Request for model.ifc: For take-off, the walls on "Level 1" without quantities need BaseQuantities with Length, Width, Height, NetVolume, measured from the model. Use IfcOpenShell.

First a look at what the model holds.

```python
import ifcopenshell
import ifcopenshell.util.element
import ifcopenshell.util.unit

model = ifcopenshell.open("model.ifc")
print(model.schema)
for unit_type in ("LENGTHUNIT", "AREAUNIT", "VOLUMEUNIT"):
    print(unit_type, ifcopenshell.util.unit.calculate_unit_scale(model, unit_type))
storey = next(s for s in model.by_type("IfcBuildingStorey") if s.Name == "Level 1")
walls = [e for e in ifcopenshell.util.element.get_decomposition(storey) if e.is_a("IfcWall")]
for e in sorted(walls, key=lambda e: e.id()):
    print(e.id(), e.is_a(), e.Name, list(ifcopenshell.util.element.get_psets(e, qtos_only=True)), sep=" | ")
```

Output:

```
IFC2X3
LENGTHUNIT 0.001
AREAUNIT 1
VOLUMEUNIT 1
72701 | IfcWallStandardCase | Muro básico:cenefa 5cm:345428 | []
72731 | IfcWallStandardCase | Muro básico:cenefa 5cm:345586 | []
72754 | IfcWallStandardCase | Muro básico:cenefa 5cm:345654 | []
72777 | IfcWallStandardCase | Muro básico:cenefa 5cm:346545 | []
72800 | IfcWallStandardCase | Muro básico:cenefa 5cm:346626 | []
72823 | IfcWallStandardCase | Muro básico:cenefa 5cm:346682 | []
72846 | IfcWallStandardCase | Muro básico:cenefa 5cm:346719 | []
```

```python
import ifcopenshell
import ifcopenshell.api.pset
import ifcopenshell.geom
import ifcopenshell.util.element
import ifcopenshell.util.shape
import ifcopenshell.util.unit

model = ifcopenshell.open("model.ifc")
unit_scale = ifcopenshell.util.unit.calculate_unit_scale(model)
volume_scale = ifcopenshell.util.unit.calculate_unit_scale(model, "VOLUMEUNIT")
settings = ifcopenshell.geom.settings()

storey = next(s for s in model.by_type("IfcBuildingStorey") if s.Name == "Level 1")
walls = [e for e in ifcopenshell.util.element.get_decomposition(storey) if e.is_a("IfcWall")]

for e in sorted(walls, key=lambda e: e.id()):
    if ifcopenshell.util.element.get_psets(e, qtos_only=True, should_inherit=False):
        continue
    # Geometry comes back in metres, in the element's own axes.
    shape = ifcopenshell.geom.create_shape(settings, e)
    values = {
        "Length": ifcopenshell.util.shape.get_x(shape.geometry) / unit_scale,
        "Width": ifcopenshell.util.shape.get_y(shape.geometry) / unit_scale,
        "Height": ifcopenshell.util.shape.get_z(shape.geometry) / unit_scale,
        "NetVolume": ifcopenshell.util.shape.get_volume(shape.geometry) / volume_scale,
    }
    qto = ifcopenshell.api.pset.add_qto(model, product=e, name="BaseQuantities")
    ifcopenshell.api.pset.edit_qto(model, qto=qto, properties=values)
    print(e.id(), {k: round(v, 3) for k, v in values.items()})

model.write("model_v2.ifc")
```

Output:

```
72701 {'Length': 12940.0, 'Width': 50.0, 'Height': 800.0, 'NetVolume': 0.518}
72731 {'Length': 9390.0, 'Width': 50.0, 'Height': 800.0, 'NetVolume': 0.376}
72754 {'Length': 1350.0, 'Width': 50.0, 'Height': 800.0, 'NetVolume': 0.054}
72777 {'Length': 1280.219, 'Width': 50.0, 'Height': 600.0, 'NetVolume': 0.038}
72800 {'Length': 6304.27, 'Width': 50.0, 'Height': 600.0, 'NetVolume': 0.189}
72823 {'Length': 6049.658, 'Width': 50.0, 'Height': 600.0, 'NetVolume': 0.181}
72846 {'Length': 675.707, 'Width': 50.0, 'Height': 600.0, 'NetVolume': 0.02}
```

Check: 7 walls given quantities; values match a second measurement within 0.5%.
